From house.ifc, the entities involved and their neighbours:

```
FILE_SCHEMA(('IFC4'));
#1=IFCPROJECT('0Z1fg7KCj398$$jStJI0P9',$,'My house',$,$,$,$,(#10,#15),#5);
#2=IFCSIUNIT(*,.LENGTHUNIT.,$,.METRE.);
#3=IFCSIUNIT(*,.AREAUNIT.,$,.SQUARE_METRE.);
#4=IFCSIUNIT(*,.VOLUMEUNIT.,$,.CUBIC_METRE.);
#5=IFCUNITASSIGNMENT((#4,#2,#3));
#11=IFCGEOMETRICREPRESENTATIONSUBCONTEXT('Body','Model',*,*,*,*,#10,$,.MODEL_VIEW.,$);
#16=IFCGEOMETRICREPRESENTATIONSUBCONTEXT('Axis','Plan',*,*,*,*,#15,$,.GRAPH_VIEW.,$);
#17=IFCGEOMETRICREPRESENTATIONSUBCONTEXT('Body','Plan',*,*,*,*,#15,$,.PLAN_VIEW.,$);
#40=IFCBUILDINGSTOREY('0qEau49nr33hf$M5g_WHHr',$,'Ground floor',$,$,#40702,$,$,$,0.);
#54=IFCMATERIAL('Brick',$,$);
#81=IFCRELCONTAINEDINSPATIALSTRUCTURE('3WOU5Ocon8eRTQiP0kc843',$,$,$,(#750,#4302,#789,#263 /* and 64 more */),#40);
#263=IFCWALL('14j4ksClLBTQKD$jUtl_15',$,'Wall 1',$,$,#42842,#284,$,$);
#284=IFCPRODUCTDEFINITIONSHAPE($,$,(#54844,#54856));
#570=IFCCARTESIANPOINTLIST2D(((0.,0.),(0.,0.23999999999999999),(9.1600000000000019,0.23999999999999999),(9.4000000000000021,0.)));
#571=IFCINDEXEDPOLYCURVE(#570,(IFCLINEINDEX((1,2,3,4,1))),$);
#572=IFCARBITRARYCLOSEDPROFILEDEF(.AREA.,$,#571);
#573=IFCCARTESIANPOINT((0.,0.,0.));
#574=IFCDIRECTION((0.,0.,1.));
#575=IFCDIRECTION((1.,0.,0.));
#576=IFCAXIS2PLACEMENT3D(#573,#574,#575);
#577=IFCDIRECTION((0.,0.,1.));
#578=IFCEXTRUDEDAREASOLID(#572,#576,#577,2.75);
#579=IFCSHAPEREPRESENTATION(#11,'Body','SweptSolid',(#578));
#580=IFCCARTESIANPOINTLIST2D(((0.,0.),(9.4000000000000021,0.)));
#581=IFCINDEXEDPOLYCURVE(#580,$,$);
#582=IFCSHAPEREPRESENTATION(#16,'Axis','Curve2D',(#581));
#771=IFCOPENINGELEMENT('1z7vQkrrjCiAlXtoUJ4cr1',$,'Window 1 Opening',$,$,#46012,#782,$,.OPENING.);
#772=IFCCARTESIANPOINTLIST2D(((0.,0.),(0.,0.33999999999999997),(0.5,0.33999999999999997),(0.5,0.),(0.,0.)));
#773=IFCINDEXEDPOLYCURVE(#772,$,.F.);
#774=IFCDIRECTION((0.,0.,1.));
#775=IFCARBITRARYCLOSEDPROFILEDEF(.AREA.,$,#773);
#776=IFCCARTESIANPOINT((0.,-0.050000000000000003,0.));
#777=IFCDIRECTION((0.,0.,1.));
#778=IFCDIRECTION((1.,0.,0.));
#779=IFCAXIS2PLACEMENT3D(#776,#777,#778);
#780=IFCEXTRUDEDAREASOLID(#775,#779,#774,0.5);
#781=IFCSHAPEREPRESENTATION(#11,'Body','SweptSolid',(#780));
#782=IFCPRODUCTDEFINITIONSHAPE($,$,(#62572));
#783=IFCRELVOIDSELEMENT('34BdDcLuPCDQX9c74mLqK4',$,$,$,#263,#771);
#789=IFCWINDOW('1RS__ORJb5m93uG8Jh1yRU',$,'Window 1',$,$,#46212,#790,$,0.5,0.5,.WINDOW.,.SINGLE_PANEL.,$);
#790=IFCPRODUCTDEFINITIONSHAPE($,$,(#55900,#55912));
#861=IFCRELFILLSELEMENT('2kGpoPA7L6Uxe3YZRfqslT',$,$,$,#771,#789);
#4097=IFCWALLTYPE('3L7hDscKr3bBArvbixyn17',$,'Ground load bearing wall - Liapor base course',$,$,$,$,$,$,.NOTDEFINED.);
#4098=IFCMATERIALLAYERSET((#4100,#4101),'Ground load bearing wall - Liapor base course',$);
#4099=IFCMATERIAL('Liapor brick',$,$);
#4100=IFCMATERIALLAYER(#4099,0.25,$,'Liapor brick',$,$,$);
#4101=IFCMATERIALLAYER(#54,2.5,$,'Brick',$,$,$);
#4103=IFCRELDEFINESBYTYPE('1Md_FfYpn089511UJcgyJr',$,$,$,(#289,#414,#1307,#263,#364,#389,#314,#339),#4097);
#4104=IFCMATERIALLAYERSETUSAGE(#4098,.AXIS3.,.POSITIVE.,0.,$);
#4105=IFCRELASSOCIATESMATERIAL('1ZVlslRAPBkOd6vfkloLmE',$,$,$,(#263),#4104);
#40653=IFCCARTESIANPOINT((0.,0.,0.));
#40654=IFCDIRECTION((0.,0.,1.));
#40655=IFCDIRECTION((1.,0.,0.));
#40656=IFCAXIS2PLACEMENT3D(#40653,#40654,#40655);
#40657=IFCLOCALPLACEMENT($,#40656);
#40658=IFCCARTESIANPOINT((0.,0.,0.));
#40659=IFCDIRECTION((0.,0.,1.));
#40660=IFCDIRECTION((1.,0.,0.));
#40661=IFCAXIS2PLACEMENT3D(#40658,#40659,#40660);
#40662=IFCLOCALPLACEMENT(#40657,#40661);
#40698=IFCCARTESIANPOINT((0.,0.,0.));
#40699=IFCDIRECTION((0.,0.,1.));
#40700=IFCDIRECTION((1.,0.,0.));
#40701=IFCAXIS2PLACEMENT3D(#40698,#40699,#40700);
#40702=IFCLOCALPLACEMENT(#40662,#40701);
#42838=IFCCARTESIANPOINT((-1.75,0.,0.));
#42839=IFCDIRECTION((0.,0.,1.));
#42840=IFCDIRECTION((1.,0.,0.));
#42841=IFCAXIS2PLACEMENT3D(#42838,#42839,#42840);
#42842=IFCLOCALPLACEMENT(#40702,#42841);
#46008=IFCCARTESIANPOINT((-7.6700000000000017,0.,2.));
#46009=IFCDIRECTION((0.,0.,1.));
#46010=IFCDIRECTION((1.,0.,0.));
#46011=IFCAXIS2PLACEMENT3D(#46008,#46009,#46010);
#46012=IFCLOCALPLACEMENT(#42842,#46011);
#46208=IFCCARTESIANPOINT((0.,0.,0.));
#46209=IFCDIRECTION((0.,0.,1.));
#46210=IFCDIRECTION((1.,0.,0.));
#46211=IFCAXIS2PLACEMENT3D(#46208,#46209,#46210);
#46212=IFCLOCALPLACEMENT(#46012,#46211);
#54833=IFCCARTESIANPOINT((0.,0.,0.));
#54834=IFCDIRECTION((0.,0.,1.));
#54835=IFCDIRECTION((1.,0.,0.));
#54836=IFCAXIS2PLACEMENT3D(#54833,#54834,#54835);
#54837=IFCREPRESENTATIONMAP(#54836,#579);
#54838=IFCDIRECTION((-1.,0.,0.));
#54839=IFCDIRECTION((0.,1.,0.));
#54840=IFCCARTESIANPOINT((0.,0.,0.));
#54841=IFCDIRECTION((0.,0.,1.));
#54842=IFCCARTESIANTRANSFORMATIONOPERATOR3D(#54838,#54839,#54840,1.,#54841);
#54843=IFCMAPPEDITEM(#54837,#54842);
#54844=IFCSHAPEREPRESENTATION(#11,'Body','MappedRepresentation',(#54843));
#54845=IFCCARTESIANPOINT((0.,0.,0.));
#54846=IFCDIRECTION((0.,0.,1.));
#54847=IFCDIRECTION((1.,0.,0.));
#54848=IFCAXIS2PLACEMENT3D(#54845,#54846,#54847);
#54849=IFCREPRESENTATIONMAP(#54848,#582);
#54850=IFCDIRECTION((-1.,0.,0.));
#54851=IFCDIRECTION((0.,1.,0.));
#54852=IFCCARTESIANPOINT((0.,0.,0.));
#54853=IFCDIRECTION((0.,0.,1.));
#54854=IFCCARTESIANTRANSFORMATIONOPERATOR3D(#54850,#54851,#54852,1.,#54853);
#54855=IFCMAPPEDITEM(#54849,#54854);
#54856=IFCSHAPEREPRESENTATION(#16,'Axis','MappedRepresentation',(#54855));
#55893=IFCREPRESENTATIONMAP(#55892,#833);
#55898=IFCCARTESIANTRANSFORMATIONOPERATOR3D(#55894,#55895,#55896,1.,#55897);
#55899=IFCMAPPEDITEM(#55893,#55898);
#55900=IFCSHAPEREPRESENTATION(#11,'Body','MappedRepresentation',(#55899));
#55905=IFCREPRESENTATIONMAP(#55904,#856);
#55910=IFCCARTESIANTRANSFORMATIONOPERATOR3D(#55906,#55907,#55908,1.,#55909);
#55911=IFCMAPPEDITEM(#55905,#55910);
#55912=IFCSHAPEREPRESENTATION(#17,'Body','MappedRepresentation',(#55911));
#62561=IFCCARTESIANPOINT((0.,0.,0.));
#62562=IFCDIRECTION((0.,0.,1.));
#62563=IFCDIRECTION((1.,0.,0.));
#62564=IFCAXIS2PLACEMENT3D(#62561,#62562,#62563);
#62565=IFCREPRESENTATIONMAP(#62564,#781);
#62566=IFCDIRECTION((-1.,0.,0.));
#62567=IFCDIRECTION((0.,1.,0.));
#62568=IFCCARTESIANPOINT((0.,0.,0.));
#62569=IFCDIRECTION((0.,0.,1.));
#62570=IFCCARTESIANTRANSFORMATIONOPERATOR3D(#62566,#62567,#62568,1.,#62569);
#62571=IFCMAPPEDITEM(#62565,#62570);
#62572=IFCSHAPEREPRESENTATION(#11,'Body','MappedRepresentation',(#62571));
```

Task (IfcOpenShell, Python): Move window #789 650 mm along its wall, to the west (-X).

```python
import ifcopenshell
import ifcopenshell.api.geometry
import ifcopenshell.util.placement
import ifcopenshell.util.unit

model = ifcopenshell.open("house.ifc")
unit_scale = ifcopenshell.util.unit.calculate_unit_scale(model)

window = model.by_guid("1RS__ORJb5m93uG8Jh1yRU")
opening = window.FillsVoids[0].RelatingOpeningElement
wall = opening.VoidsElements[0].RelatingBuildingElement

wall_matrix = ifcopenshell.util.placement.get_local_placement(wall.ObjectPlacement)
shift = wall_matrix[:3, 0] * -0.65 / unit_scale
before = ifcopenshell.util.placement.get_local_placement(window.ObjectPlacement)[:3, 3].copy()

# The window is placed relative to its opening, so it follows when the opening moves.
matrix = ifcopenshell.util.placement.get_local_placement(opening.ObjectPlacement)
matrix[:3, 3] += shift
ifcopenshell.api.geometry.edit_object_placement(
    model, product=opening, matrix=matrix, is_si=False, should_transform_children=True
)

after = ifcopenshell.util.placement.get_local_placement(window.ObjectPlacement)[:3, 3]
print("window moved by", (after - before).round(3) + 0.0)

model.write("house_v2.ifc")
```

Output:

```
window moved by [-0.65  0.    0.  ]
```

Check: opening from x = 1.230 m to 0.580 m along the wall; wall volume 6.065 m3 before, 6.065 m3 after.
